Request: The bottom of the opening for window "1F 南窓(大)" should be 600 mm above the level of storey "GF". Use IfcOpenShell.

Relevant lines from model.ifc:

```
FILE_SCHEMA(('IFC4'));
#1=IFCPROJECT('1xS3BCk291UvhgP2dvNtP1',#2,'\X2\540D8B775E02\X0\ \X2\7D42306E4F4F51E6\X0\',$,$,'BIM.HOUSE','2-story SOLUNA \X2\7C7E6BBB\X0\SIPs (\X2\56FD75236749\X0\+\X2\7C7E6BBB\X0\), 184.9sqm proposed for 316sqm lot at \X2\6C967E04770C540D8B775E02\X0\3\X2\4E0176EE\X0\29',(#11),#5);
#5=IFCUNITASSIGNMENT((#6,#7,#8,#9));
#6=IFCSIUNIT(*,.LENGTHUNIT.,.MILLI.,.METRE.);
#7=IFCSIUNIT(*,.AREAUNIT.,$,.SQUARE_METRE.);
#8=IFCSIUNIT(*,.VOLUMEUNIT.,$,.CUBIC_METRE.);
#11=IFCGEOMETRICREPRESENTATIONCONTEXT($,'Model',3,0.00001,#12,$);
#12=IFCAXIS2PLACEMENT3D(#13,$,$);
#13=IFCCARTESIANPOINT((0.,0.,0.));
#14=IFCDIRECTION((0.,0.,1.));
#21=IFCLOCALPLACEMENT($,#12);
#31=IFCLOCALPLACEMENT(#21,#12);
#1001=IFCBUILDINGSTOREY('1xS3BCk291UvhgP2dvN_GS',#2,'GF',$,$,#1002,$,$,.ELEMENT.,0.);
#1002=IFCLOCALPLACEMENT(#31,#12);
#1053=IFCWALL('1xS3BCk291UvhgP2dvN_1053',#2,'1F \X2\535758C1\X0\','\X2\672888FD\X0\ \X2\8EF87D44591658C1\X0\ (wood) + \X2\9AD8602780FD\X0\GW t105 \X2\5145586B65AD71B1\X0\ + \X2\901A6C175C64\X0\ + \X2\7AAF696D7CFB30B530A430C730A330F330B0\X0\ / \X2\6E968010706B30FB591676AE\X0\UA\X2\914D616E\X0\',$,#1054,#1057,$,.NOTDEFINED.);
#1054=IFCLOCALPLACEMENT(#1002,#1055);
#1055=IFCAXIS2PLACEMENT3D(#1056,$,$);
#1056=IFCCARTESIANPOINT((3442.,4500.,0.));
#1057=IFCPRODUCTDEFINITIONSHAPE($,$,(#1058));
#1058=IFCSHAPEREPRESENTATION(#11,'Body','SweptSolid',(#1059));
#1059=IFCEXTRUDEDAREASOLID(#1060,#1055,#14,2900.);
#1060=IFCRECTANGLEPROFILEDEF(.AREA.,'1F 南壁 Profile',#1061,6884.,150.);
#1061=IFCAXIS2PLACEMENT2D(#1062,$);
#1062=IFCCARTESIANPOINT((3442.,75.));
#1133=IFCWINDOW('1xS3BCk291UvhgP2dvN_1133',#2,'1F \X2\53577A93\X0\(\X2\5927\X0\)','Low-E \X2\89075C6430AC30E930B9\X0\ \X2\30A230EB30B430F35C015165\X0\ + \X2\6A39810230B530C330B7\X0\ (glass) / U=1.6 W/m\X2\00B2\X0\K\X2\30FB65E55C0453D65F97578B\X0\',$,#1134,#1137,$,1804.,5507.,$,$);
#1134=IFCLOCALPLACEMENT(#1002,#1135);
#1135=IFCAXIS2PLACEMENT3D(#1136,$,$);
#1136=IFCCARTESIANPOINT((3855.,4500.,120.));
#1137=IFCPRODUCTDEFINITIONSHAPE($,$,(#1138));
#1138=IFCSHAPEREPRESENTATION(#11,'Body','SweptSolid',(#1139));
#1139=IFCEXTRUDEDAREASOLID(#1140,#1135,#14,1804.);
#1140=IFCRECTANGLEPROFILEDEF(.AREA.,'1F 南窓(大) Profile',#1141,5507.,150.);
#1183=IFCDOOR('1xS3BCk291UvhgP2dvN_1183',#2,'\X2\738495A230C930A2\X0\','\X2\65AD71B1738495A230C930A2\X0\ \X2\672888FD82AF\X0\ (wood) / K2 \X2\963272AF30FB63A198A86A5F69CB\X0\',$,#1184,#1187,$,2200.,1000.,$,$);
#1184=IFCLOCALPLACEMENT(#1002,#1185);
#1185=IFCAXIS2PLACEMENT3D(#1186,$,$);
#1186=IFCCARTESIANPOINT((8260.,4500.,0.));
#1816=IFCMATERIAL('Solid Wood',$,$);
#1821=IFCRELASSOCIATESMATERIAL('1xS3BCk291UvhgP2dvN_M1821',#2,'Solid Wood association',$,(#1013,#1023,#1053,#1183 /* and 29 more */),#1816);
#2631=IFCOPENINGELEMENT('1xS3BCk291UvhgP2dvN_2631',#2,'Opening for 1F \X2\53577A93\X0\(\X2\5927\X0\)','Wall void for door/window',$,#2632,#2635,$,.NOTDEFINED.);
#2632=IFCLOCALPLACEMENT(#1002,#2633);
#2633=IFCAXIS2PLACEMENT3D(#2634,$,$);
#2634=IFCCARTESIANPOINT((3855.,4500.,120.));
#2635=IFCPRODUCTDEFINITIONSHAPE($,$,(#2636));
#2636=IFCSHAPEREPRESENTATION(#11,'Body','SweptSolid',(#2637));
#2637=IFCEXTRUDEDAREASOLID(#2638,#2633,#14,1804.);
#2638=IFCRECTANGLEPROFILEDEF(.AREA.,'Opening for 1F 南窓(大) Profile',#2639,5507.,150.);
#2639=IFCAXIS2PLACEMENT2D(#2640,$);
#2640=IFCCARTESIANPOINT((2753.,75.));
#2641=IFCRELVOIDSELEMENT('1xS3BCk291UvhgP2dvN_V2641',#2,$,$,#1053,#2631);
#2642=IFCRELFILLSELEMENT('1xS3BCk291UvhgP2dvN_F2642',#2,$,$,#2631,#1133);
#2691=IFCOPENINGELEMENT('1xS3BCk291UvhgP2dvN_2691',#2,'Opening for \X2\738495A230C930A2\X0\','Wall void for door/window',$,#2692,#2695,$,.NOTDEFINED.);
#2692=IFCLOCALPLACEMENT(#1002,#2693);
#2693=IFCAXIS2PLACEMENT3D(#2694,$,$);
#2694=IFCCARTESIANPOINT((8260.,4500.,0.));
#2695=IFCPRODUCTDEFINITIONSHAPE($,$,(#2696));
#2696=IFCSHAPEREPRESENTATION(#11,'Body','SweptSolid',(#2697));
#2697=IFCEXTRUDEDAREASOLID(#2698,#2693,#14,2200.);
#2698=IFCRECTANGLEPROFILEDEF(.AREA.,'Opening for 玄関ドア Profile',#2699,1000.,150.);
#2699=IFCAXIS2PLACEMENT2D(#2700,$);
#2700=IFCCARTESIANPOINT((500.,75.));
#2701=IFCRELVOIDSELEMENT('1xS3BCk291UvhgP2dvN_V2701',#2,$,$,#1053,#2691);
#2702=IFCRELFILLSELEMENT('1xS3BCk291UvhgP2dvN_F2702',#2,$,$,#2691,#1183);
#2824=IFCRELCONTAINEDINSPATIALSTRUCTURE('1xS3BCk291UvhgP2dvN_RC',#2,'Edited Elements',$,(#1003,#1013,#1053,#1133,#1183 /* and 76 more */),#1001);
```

```python
import numpy as np
import ifcopenshell
import ifcopenshell.api.geometry
import ifcopenshell.geom
import ifcopenshell.util.element
import ifcopenshell.util.placement
import ifcopenshell.util.shape
import ifcopenshell.util.unit

model = ifcopenshell.open("model.ifc")
unit_scale = ifcopenshell.util.unit.calculate_unit_scale(model)

window = model.by_guid("1xS3BCk291UvhgP2dvN_1133")
opening = window.FillsVoids[0].RelatingOpeningElement
storey = ifcopenshell.util.element.get_container(window, ifc_class="IfcBuildingStorey")
level = ifcopenshell.util.placement.get_local_placement(storey.ObjectPlacement)[2, 3]

# The opening's origin need not be at the sill, so measure its lowest point.
shape = ifcopenshell.geom.create_shape(ifcopenshell.geom.settings(), opening)
bottom = ifcopenshell.util.shape.get_shape_bottom_elevation(shape, shape.geometry) / unit_scale
dz = level + 0.6 / unit_scale - bottom

shift = np.array([0.0, 0.0, dz])
# The window is not placed relative to its opening, so move both.
for product in (opening, window):
    matrix = ifcopenshell.util.placement.get_local_placement(product.ObjectPlacement)
    matrix[:3, 3] += shift
    ifcopenshell.api.geometry.edit_object_placement(model, product=product, matrix=matrix, is_si=False)

print(f"moved by {dz * unit_scale:+.3f} m")

model.write("model-out.ifc")
```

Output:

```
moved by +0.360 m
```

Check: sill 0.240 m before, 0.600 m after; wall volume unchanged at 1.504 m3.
